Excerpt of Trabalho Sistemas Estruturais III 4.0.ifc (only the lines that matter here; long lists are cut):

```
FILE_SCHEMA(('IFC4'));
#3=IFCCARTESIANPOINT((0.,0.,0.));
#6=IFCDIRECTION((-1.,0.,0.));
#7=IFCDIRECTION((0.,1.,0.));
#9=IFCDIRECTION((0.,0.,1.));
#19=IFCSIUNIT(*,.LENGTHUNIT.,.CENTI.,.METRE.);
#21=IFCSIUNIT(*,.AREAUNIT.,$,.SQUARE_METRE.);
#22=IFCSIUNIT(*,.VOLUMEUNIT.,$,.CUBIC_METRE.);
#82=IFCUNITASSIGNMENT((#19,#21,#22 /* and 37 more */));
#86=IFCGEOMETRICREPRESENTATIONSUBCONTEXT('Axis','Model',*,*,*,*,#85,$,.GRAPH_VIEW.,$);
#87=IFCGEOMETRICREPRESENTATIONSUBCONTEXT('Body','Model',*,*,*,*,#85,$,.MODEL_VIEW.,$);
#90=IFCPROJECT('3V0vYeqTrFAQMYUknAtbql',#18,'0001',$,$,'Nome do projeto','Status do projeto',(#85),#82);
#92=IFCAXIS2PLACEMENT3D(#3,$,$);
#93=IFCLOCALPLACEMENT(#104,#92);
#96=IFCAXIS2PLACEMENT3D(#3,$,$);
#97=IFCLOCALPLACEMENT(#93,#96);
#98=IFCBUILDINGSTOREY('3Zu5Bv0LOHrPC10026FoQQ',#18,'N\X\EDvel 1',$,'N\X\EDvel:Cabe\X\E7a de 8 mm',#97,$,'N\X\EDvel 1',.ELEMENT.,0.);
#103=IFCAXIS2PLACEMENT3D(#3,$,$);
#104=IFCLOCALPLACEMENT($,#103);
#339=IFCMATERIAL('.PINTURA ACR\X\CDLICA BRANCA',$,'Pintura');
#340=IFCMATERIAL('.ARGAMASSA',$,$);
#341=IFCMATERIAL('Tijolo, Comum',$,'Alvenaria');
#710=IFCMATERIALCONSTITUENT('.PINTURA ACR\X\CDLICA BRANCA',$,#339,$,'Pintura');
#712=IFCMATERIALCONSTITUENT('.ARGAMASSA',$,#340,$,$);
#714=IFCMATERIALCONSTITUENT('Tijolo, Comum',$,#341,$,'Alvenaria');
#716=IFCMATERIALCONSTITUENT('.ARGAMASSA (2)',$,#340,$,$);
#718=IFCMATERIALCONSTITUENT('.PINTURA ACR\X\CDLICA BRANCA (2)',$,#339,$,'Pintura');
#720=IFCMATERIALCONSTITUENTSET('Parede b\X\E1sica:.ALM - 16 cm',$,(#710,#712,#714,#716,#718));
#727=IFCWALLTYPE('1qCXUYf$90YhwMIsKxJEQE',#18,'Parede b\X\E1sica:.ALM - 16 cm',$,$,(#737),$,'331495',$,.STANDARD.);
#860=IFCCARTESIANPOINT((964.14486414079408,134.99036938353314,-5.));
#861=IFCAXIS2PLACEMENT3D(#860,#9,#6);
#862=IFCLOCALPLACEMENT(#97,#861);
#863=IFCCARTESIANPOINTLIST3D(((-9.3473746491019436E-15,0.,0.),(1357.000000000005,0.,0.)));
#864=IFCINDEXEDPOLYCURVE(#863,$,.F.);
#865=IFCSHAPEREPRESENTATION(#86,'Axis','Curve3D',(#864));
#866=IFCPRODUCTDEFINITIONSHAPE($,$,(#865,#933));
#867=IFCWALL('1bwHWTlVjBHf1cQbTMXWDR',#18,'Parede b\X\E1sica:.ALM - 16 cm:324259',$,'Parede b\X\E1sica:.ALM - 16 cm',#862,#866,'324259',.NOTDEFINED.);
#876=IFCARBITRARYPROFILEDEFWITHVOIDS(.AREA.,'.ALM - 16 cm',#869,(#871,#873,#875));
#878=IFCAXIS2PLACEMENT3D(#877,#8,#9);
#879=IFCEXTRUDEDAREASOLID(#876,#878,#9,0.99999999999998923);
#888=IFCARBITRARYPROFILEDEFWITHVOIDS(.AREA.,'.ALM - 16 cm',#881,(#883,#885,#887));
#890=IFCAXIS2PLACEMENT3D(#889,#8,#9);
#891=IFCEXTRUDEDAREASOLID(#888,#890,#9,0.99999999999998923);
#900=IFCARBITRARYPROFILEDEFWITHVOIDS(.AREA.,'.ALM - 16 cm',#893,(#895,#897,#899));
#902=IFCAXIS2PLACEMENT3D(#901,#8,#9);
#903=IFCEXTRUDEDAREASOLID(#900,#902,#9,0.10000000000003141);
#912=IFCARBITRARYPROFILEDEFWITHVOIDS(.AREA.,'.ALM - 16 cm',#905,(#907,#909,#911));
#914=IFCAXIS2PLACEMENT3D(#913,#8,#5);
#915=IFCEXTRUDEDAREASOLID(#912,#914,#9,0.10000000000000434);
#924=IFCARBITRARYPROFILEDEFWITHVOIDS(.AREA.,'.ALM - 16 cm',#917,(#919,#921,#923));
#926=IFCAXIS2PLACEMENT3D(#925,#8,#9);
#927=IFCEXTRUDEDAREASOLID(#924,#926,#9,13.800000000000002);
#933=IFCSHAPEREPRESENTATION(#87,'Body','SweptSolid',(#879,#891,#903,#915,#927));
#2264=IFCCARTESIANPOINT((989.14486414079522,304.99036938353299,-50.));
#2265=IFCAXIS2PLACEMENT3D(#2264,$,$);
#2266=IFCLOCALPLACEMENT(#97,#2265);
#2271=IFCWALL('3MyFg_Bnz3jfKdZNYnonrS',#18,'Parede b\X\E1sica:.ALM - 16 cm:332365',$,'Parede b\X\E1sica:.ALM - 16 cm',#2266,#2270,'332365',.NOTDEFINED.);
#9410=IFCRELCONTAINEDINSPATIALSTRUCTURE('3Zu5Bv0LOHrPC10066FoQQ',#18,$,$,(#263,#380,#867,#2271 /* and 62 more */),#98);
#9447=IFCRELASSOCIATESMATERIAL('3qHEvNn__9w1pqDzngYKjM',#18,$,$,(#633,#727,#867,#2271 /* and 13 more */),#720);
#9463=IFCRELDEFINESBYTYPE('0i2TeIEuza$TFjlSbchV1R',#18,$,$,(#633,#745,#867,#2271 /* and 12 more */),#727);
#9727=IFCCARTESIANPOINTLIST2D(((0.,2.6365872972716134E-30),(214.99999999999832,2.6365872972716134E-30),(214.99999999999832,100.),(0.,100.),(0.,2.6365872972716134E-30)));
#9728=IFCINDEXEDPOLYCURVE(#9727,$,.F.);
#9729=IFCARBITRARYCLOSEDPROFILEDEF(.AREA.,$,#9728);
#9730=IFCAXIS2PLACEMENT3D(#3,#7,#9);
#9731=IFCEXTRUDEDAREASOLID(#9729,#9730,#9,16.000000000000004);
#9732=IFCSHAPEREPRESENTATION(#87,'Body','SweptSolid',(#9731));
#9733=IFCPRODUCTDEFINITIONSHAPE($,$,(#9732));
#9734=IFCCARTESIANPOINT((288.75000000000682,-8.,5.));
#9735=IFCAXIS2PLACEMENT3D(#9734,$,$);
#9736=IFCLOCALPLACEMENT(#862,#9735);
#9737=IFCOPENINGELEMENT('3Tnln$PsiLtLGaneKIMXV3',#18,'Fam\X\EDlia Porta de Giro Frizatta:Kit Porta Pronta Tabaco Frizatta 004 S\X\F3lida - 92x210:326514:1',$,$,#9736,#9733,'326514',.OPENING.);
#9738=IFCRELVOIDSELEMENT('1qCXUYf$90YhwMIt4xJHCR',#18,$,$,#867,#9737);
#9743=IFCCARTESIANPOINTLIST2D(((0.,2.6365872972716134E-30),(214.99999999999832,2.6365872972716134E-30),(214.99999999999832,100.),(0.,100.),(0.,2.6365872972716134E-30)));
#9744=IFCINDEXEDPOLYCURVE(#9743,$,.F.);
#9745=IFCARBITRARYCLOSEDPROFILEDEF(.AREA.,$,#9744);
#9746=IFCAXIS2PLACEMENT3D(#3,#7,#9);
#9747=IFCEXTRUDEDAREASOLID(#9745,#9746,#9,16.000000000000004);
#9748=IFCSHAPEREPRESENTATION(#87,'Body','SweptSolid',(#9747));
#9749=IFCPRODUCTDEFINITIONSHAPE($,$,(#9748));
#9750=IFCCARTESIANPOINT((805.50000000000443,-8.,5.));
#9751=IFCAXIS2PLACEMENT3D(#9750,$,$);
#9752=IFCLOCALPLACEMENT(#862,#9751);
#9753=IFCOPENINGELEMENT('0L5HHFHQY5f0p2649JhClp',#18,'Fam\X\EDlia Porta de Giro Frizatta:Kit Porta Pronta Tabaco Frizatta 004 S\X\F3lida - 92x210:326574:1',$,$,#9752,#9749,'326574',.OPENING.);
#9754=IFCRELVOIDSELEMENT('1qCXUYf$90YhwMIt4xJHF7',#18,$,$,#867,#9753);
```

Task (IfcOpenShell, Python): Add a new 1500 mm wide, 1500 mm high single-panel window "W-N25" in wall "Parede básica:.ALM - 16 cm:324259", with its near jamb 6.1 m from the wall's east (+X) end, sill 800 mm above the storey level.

```python
import numpy as np
import ifcopenshell
import ifcopenshell.api.feature
import ifcopenshell.api.geometry
import ifcopenshell.api.root
import ifcopenshell.api.spatial
import ifcopenshell.geom
import ifcopenshell.util.element
import ifcopenshell.util.placement
import ifcopenshell.util.representation
import ifcopenshell.util.shape
import ifcopenshell.util.unit

model = ifcopenshell.open("Trabalho Sistemas Estruturais III 4.0.ifc")
unit_scale = ifcopenshell.util.unit.calculate_unit_scale(model)
settings = ifcopenshell.geom.settings()


def volume(element):
    """Net volume in cubic metres, openings subtracted."""
    shape = ifcopenshell.geom.create_shape(settings, element)
    return ifcopenshell.util.shape.get_volume(shape.geometry)


wall = model.by_id(867)
storey = ifcopenshell.util.element.get_container(wall, ifc_class="IfcBuildingStorey")
context = ifcopenshell.util.representation.get_context(model, "Model", "Body", "MODEL_VIEW")
before = volume(wall)

width, height, from_end, sill = 1.5, 1.5, 6.1, 0.8  # metres

# The wall runs along its own X axis, and the end named is its -X end.
wall_shape = ifcopenshell.geom.create_shape(settings, wall)
x, y, z = ifcopenshell.util.shape.get_vertices(wall_shape.geometry).T
start = x.min() + from_end
face, thickness = float(y.min()), float(y.max() - y.min())
wall_matrix = ifcopenshell.util.placement.get_local_placement(wall.ObjectPlacement)
level = ifcopenshell.util.placement.get_local_placement(storey.ObjectPlacement)[2, 3]


def in_wall(x, y):
    """Placement at x, y metres in the wall's axes, at sill height."""
    matrix = wall_matrix.copy()
    matrix[:, 3] = wall_matrix @ np.array([x / unit_scale, y / unit_scale, 0.0, 1.0])
    matrix[2, 3] = level + sill / unit_scale
    return matrix


# Opening: a box that overshoots both wall faces by 50 mm.
opening = ifcopenshell.api.root.create_entity(model, ifc_class="IfcOpeningElement", predefined_type="OPENING")
box = ifcopenshell.api.geometry.add_wall_representation(
    model, context=context, length=width, height=height, thickness=thickness + 0.1
)
ifcopenshell.api.geometry.assign_representation(model, product=opening, representation=box)
ifcopenshell.api.geometry.edit_object_placement(model, product=opening, matrix=in_wall(start, face - 0.05), is_si=False)
ifcopenshell.api.feature.add_feature(model, feature=opening, element=wall)

window = ifcopenshell.api.root.create_entity(model, ifc_class="IfcWindow", name="W-N25", predefined_type="WINDOW")
window.OverallWidth, window.OverallHeight = width / unit_scale, height / unit_scale
window.PartitioningType = "SINGLE_PANEL"
body = ifcopenshell.api.geometry.add_window_representation(
    model,
    context=context,
    overall_width=window.OverallWidth,
    overall_height=window.OverallHeight,
    partition_type="SINGLE_PANEL",
)
ifcopenshell.api.geometry.assign_representation(model, product=window, representation=body)
ifcopenshell.api.spatial.assign_container(model, products=[window], relating_structure=storey)
ifcopenshell.api.feature.add_filling(model, opening=opening, element=window)

# Centre the window in the wall's thickness.
ifcopenshell.api.geometry.edit_object_placement(model, product=window, matrix=in_wall(start, face), is_si=False)
window_shape = ifcopenshell.geom.create_shape(settings, window)
depth = ifcopenshell.util.shape.get_vertices(window_shape.geometry)[:, 1]
offset = face + thickness / 2 - (depth.min() + depth.max()) / 2
ifcopenshell.api.geometry.edit_object_placement(model, product=window, matrix=in_wall(start, offset), is_si=False)

after = volume(wall)

print(f"wall volume {before:.3f} -> {after:.3f} m3")

model.write("Trabalho Sistemas Estruturais III 4.0-out.ifc")
```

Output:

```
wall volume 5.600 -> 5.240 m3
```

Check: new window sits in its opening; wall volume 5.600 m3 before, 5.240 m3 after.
